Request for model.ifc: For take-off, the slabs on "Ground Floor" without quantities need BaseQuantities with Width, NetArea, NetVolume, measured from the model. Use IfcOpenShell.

First a look at what the model holds.

```python
import ifcopenshell
import ifcopenshell.util.element
import ifcopenshell.util.unit

model = ifcopenshell.open("model.ifc")
print(model.schema)
for unit_type in ("LENGTHUNIT", "AREAUNIT", "VOLUMEUNIT"):
    print(unit_type, ifcopenshell.util.unit.calculate_unit_scale(model, unit_type))
storey = next(s for s in model.by_type("IfcBuildingStorey") if s.Name == "Ground Floor")
slabs = [e for e in ifcopenshell.util.element.get_decomposition(storey) if e.is_a("IfcSlab")]
for e in sorted(slabs, key=lambda e: e.id()):
    print(e.id(), e.is_a(), e.Name, list(ifcopenshell.util.element.get_psets(e, qtos_only=True)), sep=" | ")
```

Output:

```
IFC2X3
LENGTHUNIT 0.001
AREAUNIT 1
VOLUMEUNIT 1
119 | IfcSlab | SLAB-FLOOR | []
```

```python
import ifcopenshell
import ifcopenshell.api.pset
import ifcopenshell.geom
import ifcopenshell.util.element
import ifcopenshell.util.shape
import ifcopenshell.util.unit

model = ifcopenshell.open("model.ifc")
unit_scale = ifcopenshell.util.unit.calculate_unit_scale(model)
area_scale = ifcopenshell.util.unit.calculate_unit_scale(model, "AREAUNIT")
volume_scale = ifcopenshell.util.unit.calculate_unit_scale(model, "VOLUMEUNIT")
settings = ifcopenshell.geom.settings()

storey = next(s for s in model.by_type("IfcBuildingStorey") if s.Name == "Ground Floor")
slabs = [e for e in ifcopenshell.util.element.get_decomposition(storey) if e.is_a("IfcSlab")]

for e in sorted(slabs, key=lambda e: e.id()):
    if ifcopenshell.util.element.get_psets(e, qtos_only=True, should_inherit=False):
        continue
    # Geometry comes back in metres, in the element's own axes.
    shape = ifcopenshell.geom.create_shape(settings, e)
    values = {
        "Width": ifcopenshell.util.shape.get_z(shape.geometry) / unit_scale,
        "NetArea": ifcopenshell.util.shape.get_footprint_area(shape.geometry) / area_scale,
        "NetVolume": ifcopenshell.util.shape.get_volume(shape.geometry) / volume_scale,
    }
    qto = ifcopenshell.api.pset.add_qto(model, product=e, name="BaseQuantities")
    ifcopenshell.api.pset.edit_qto(model, qto=qto, properties=values)
    print(e.id(), {k: round(v, 3) for k, v in values.items()})

model.write("model_rev.ifc")
```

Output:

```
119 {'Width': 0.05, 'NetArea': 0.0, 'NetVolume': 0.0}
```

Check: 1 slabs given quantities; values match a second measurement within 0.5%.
